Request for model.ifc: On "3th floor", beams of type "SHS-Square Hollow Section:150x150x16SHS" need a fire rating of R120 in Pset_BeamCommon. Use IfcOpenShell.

First a look at what the model holds.

```python
import ifcopenshell
import ifcopenshell.util.element

model = ifcopenshell.open("model.ifc")
print(model.schema)
storey = next(s for s in model.by_type("IfcBuildingStorey") if s.Name == "3th floor")
beams = [e for e in ifcopenshell.util.element.get_decomposition(storey) if e.is_a("IfcBeam")]
seen = {}
for e in beams:
    element_type = ifcopenshell.util.element.get_type(e)
    key = (element_type.Name if element_type != e and element_type else None, ifcopenshell.util.element.get_pset(e, "Pset_BeamCommon", "FireRating"))
    seen[key] = seen.get(key, 0) + 1
for (name, value), count in sorted(seen.items(), key=str):
    print(count, "x", name, "|", value)
```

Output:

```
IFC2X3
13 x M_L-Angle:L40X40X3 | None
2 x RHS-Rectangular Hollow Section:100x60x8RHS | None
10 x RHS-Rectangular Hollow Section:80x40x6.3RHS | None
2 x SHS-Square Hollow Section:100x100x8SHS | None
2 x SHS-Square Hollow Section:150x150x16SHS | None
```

```python
import ifcopenshell
import ifcopenshell.api.pset
import ifcopenshell.util.element

model = ifcopenshell.open("model.ifc")

storey = next(s for s in model.by_type("IfcBuildingStorey") if s.Name == "3th floor")
beams = [e for e in ifcopenshell.util.element.get_decomposition(storey) if e.is_a("IfcBeam")]

count = 0
for e in beams:
    element_type = ifcopenshell.util.element.get_type(e)
    if element_type in (None, e) or element_type.Name != "SHS-Square Hollow Section:150x150x16SHS":
        continue
    # add_pset returns the element's existing set when there is one.
    pset = ifcopenshell.api.pset.add_pset(model, product=e, name="Pset_BeamCommon")
    ifcopenshell.api.pset.edit_pset(model, pset=pset, properties={"FireRating": "R120"})
    count += 1

print(count, "beams updated")

model.write("model_edited.ifc")
```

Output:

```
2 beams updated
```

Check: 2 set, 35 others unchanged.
